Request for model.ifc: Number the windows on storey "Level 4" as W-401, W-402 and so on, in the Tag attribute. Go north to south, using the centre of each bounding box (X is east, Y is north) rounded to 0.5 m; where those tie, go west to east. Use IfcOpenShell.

First a look at what the model holds.

```python
import ifcopenshell
import ifcopenshell.util.element
import ifcopenshell.util.placement

model = ifcopenshell.open("model.ifc")
print(model.schema)
storey = next(s for s in model.by_type("IfcBuildingStorey") if s.Name == "Level 4")
windows = [e for e in ifcopenshell.util.element.get_decomposition(storey) if e.is_a("IfcWindow")]
for e in sorted(windows, key=lambda e: e.id()):
    origin = ifcopenshell.util.placement.get_local_placement(e.ObjectPlacement)[:3, 3]
    print(e.id(), e.Tag, e.Name, origin.round(2) + 0.0, sep=" | ")
```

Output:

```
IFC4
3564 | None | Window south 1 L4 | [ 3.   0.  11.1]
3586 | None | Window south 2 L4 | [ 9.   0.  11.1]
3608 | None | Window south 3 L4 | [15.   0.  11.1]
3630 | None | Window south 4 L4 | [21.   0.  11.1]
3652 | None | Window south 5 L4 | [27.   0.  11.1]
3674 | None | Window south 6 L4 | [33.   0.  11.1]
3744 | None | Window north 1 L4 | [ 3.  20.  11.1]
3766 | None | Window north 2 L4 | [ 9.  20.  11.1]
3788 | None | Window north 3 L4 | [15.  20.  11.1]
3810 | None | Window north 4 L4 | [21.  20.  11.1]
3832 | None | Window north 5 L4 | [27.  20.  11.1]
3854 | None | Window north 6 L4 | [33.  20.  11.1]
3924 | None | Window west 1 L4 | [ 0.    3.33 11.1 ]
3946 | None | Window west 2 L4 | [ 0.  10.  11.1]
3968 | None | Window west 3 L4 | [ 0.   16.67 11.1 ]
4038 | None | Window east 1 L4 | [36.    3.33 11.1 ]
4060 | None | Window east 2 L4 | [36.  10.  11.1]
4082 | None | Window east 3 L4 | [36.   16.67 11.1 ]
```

```python
import ifcopenshell
import ifcopenshell.geom
import ifcopenshell.util.element
import ifcopenshell.util.shape

model = ifcopenshell.open("model.ifc")
settings = ifcopenshell.geom.settings()
settings.set("use-world-coords", True)


def centre(element):
    shape = ifcopenshell.geom.create_shape(settings, element)
    return ifcopenshell.util.shape.get_bbox_centroid(shape.geometry)


storey = next(s for s in model.by_type("IfcBuildingStorey") if s.Name == "Level 4")
windows = [e for e in ifcopenshell.util.element.get_decomposition(storey) if e.is_a("IfcWindow")]

# Insertion points can sit at a corner or the storey origin, so sort by the geometry (in metres).
centres = {e: centre(e) for e in windows}
windows.sort(key=lambda e: (-round(centres[e][1] / 0.5), centres[e][0]))

for i, e in enumerate(windows, start=1):
    number = f"W-4{i:02d}"
    e.Tag = number
    print(e.id(), number)

model.write("model-out.ifc")
```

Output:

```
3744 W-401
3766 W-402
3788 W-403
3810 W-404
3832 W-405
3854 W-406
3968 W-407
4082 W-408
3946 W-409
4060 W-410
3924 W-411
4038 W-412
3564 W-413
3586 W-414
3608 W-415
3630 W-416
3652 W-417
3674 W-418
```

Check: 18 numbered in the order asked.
